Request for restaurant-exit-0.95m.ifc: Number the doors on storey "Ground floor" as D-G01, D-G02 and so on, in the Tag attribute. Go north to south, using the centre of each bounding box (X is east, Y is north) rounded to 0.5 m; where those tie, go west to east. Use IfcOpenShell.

First a look at what the model holds.

```python
import ifcopenshell
import ifcopenshell.util.element
import ifcopenshell.util.placement

model = ifcopenshell.open("restaurant-exit-0.95m.ifc")
print(model.schema)
storey = next(s for s in model.by_type("IfcBuildingStorey") if s.Name == "Ground floor")
doors = [e for e in ifcopenshell.util.element.get_decomposition(storey) if e.is_a("IfcDoor")]
for e in sorted(doors, key=lambda e: e.id()):
    origin = ifcopenshell.util.placement.get_local_placement(e.ObjectPlacement)[:3, 3]
    print(e.id(), e.Tag, e.Name, origin.round(2) + 0.0, sep=" | ")
```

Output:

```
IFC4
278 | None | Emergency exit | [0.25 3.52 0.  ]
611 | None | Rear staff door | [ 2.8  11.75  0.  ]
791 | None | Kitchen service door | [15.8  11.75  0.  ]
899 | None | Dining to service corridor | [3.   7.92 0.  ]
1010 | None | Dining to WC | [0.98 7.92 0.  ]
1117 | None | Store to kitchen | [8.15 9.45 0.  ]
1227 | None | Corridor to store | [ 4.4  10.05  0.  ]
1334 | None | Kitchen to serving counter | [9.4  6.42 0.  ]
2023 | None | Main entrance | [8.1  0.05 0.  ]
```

```python
import ifcopenshell
import ifcopenshell.geom
import ifcopenshell.util.element
import ifcopenshell.util.shape

model = ifcopenshell.open("restaurant-exit-0.95m.ifc")
settings = ifcopenshell.geom.settings()
settings.set("use-world-coords", True)


def centre(element):
    shape = ifcopenshell.geom.create_shape(settings, element)
    return ifcopenshell.util.shape.get_bbox_centroid(shape.geometry)


storey = next(s for s in model.by_type("IfcBuildingStorey") if s.Name == "Ground floor")
doors = [e for e in ifcopenshell.util.element.get_decomposition(storey) if e.is_a("IfcDoor")]

# Insertion points can sit at a corner or the storey origin, so sort by the geometry (in metres).
centres = {e: centre(e) for e in doors}
doors.sort(key=lambda e: (-round(centres[e][1] / 0.5), centres[e][0]))

for i, e in enumerate(doors, start=1):
    number = f"D-G{i:02d}"
    e.Tag = number
    print(e.id(), number)

model.write("restaurant-exit-0.95m_edited.ifc")
```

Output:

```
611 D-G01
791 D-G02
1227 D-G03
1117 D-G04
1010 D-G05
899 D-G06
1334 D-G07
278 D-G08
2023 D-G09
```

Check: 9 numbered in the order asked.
